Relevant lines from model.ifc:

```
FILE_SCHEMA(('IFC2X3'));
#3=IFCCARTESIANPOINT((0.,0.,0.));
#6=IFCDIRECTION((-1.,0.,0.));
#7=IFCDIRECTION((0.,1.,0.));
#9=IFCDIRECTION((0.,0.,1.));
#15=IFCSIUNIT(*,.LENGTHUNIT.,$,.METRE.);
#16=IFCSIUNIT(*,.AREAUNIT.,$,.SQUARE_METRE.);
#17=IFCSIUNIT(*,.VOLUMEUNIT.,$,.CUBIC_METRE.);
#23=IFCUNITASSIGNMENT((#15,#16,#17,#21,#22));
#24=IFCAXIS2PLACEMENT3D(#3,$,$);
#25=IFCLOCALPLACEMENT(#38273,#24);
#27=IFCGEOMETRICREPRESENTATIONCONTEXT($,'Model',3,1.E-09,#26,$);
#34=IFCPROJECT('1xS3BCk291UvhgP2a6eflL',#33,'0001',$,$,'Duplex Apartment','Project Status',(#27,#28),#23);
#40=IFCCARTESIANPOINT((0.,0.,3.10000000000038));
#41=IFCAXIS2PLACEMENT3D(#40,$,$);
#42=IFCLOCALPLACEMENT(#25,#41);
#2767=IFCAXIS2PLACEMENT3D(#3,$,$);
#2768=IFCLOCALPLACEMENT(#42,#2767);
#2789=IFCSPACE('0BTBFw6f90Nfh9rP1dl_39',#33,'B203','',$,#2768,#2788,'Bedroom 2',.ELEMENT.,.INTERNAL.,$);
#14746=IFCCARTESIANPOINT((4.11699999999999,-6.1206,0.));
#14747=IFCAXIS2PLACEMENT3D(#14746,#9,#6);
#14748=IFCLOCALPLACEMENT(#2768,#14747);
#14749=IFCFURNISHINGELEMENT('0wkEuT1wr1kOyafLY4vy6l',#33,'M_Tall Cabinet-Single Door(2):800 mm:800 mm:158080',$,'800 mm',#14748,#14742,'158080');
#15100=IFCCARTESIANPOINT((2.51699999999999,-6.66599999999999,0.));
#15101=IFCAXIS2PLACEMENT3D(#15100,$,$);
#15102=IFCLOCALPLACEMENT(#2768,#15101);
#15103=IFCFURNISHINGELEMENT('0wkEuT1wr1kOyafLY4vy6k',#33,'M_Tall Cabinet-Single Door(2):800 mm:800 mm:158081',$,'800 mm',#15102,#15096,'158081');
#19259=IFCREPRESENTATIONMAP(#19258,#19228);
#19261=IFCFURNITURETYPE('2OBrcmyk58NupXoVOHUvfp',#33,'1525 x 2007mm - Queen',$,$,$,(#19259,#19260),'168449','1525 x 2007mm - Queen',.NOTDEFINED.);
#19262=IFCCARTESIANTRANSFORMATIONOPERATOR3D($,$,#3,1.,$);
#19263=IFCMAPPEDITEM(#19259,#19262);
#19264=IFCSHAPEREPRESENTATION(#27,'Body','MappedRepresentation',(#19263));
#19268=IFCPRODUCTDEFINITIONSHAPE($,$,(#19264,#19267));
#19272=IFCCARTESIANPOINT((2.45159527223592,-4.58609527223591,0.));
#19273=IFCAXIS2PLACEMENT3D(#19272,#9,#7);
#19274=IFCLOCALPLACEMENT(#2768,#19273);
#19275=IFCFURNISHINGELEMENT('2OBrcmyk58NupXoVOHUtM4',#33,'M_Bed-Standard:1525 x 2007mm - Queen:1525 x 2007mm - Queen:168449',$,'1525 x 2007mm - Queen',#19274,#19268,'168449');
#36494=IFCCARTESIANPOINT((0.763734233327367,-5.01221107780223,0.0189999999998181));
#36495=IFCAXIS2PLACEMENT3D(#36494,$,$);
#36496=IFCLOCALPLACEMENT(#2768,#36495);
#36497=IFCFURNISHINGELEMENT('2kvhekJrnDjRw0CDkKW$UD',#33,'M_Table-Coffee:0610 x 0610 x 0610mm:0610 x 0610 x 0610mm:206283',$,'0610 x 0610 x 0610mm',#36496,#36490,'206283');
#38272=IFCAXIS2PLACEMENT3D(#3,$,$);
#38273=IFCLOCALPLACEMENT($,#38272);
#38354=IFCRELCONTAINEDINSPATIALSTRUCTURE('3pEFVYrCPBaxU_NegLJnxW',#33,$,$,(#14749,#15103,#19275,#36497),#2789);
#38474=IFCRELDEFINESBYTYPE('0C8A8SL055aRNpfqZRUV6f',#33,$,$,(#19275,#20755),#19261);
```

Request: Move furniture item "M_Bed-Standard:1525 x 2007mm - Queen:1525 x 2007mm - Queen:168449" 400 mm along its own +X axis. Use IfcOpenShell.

```python
import ifcopenshell
import ifcopenshell.api.geometry
import ifcopenshell.util.placement
import ifcopenshell.util.unit

model = ifcopenshell.open("model.ifc")
unit_scale = ifcopenshell.util.unit.calculate_unit_scale(model)

item = model.by_id(19275)
matrix = ifcopenshell.util.placement.get_local_placement(item.ObjectPlacement)
matrix[:3, 3] += matrix[:3, 0] * 0.4 / unit_scale
ifcopenshell.api.geometry.edit_object_placement(model, product=item, matrix=matrix, is_si=False)

print(ifcopenshell.util.placement.get_local_placement(item.ObjectPlacement).round(3) + 0.0)

model.write("model_updated.ifc")
```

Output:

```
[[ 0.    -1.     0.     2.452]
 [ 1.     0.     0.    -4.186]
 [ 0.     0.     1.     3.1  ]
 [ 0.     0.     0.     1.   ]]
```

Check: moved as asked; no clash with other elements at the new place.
